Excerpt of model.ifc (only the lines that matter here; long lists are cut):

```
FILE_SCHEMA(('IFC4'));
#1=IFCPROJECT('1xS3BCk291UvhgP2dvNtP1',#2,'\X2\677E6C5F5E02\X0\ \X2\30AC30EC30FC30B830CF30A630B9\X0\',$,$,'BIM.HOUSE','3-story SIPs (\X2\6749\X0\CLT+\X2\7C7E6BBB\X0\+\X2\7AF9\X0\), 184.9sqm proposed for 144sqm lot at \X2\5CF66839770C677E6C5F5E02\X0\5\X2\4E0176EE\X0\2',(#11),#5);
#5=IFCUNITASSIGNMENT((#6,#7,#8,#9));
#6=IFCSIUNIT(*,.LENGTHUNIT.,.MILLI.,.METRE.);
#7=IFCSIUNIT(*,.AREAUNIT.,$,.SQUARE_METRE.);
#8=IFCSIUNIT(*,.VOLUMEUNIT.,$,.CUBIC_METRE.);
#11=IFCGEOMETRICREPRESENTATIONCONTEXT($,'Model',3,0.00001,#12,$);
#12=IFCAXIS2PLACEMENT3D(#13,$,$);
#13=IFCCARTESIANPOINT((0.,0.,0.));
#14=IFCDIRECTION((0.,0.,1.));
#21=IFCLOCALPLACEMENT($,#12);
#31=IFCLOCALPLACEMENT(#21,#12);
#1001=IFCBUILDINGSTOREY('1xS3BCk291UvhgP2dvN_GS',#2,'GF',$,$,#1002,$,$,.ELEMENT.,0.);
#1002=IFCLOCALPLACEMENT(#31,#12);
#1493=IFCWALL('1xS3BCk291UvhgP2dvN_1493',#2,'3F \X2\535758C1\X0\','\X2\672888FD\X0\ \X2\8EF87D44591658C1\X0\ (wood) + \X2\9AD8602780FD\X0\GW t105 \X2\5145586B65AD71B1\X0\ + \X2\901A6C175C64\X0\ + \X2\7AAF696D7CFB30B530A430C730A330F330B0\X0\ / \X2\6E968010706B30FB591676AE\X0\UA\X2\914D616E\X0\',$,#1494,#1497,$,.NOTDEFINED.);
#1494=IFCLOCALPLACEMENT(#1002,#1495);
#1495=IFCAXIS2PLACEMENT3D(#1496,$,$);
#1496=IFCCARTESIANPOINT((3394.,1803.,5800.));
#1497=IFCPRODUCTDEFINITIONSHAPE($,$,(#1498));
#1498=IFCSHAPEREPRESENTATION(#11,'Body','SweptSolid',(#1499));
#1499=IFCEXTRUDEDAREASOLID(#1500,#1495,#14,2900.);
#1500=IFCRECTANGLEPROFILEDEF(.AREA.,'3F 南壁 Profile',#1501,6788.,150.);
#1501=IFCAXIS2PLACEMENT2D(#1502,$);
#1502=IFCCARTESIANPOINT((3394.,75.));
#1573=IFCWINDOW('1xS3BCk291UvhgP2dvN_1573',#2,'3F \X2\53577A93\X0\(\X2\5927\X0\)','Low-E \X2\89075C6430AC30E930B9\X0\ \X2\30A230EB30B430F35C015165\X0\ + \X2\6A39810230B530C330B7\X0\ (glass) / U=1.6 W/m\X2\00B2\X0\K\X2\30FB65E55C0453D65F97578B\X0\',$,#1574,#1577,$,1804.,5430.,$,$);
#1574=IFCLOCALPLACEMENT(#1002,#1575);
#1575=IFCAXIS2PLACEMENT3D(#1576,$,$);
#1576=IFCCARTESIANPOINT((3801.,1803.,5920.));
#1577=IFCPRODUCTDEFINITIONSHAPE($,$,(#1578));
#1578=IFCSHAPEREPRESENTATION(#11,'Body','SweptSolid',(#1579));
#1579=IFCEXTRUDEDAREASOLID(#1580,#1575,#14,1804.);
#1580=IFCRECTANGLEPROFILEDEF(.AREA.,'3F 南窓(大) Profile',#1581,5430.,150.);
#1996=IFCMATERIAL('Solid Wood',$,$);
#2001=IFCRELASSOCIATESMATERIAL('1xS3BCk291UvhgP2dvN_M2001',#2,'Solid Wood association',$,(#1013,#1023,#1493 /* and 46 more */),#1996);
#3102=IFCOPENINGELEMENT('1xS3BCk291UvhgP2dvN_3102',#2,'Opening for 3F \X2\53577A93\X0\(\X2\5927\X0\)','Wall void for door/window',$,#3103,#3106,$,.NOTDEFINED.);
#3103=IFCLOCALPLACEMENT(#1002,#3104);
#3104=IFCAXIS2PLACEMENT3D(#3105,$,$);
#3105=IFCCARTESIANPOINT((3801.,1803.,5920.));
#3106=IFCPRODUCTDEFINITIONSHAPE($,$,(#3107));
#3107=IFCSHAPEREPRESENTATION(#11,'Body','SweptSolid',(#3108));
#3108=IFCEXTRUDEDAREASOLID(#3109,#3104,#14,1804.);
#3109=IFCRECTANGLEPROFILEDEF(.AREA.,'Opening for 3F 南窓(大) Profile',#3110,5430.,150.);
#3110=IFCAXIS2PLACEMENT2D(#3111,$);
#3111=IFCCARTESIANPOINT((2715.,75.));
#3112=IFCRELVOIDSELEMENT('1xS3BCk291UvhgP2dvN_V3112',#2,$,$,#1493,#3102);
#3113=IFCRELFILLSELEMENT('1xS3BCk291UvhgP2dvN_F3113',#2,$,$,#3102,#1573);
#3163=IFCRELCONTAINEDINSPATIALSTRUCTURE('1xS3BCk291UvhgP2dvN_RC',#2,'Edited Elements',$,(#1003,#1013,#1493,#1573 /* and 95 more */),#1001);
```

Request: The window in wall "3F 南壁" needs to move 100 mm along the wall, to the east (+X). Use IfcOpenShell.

```python
import ifcopenshell
import ifcopenshell.api.geometry
import ifcopenshell.util.placement

model = ifcopenshell.open("model.ifc")

window = model.by_guid("1xS3BCk291UvhgP2dvN_1573")
opening = window.FillsVoids[0].RelatingOpeningElement
wall = opening.VoidsElements[0].RelatingBuildingElement

wall_matrix = ifcopenshell.util.placement.get_local_placement(wall.ObjectPlacement)
shift = wall_matrix[:3, 0] * 100.0
before = ifcopenshell.util.placement.get_local_placement(window.ObjectPlacement)[:3, 3].copy()

# The window is not placed relative to its opening, so move both.
for product in (opening, window):
    matrix = ifcopenshell.util.placement.get_local_placement(product.ObjectPlacement)
    matrix[:3, 3] += shift
    ifcopenshell.api.geometry.edit_object_placement(model, product=product, matrix=matrix, is_si=False)

after = ifcopenshell.util.placement.get_local_placement(window.ObjectPlacement)[:3, 3]
print("window moved by", (after - before).round(3) + 0.0)

model.write("model_updated.ifc")
```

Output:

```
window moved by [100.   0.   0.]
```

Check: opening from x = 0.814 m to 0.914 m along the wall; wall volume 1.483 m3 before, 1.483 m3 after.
